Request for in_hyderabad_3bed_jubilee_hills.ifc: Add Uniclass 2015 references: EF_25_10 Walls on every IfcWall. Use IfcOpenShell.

First a look at what the model holds.

```python
import ifcopenshell

model = ifcopenshell.open("in_hyderabad_3bed_jubilee_hills.ifc")
print(model.schema)
print("classifications:", [c.Name for c in model.by_type("IfcClassification")])
for ifc_class in ("IfcDoor", "IfcRoof", "IfcStair", "IfcWall", "IfcWindow"):
    print(ifc_class, len(model.by_type(ifc_class)))
```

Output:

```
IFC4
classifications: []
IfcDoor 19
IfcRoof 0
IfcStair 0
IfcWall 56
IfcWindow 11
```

```python
import ifcopenshell
import ifcopenshell.api.classification

model = ifcopenshell.open("in_hyderabad_3bed_jubilee_hills.ifc")

system = ifcopenshell.api.classification.add_classification(model, classification="Uniclass 2015")

codes = {
    "IfcWall": ("EF_25_10", "Walls"),
}
for ifc_class, (code, name) in codes.items():
    products = model.by_type(ifc_class)
    ifcopenshell.api.classification.add_reference(
        model, products=products, classification=system, identification=code, name=name
    )
    print(code, len(products))

model.write("in_hyderabad_3bed_jubilee_hills_updated.ifc")
```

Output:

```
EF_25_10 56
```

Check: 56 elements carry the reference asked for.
